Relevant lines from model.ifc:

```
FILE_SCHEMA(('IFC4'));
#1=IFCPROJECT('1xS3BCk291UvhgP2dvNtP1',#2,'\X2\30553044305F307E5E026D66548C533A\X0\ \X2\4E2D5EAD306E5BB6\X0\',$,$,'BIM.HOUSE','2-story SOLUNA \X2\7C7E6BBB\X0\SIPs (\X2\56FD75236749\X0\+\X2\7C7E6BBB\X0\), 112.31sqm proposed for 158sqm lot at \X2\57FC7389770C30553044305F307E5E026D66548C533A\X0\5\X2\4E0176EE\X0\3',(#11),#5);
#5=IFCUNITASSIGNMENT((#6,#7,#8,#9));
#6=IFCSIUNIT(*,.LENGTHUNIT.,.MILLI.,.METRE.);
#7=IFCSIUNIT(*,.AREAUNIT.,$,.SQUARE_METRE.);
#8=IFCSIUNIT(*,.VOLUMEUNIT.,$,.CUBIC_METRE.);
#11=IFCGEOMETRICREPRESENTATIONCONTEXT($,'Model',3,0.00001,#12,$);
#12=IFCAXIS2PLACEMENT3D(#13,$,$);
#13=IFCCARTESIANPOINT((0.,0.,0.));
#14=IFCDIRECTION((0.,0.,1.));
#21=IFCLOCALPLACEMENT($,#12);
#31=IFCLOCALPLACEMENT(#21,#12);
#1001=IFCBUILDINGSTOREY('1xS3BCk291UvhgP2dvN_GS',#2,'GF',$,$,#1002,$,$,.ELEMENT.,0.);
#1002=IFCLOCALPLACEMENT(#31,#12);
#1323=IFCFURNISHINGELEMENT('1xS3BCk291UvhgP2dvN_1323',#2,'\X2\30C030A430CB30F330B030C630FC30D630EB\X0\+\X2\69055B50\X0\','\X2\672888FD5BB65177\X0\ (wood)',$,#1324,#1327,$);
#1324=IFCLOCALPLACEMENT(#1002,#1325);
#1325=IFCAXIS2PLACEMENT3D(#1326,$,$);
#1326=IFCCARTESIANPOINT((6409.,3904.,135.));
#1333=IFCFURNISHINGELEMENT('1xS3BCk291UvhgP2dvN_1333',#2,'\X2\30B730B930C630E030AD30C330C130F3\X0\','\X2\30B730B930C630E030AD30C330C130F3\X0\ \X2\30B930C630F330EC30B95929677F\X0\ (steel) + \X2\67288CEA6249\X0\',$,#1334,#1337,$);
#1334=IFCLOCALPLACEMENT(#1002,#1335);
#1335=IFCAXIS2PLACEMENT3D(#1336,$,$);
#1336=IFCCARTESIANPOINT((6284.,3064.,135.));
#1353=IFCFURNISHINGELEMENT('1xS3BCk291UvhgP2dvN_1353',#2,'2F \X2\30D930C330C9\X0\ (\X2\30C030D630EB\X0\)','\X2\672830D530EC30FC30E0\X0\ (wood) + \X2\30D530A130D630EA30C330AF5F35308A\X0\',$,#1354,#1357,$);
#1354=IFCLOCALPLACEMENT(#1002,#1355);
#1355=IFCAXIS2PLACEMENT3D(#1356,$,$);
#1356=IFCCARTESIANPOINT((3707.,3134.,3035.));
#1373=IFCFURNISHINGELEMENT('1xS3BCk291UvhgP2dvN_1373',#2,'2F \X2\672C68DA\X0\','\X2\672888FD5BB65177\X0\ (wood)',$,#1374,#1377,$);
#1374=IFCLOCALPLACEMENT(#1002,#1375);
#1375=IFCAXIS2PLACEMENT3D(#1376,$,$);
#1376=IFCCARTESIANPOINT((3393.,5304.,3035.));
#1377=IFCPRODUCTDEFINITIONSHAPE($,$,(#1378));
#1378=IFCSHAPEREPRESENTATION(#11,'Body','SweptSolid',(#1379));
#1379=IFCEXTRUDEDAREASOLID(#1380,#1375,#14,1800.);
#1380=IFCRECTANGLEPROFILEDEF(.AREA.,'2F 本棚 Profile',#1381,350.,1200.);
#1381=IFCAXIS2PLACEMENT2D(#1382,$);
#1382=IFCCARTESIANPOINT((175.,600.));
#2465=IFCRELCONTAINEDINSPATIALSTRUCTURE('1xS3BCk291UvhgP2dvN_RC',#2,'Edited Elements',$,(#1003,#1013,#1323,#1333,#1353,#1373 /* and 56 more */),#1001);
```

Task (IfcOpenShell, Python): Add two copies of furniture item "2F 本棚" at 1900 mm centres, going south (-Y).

```python
import numpy as np
import ifcopenshell
import ifcopenshell.api.geometry
import ifcopenshell.api.root
import ifcopenshell.util.element
import ifcopenshell.util.placement
import ifcopenshell.util.unit

model = ifcopenshell.open("model.ifc")
unit_scale = ifcopenshell.util.unit.calculate_unit_scale(model)


def reuse_history(source, copy):
    """copy_class also copies each property set's owner history, people and application; keep the originals."""
    for rel in copy.IsDefinedBy:
        if rel.is_a("IfcRelDefinesByProperties") and (history := rel.RelatingPropertyDefinition.OwnerHistory):
            rel.RelatingPropertyDefinition.OwnerHistory = source.OwnerHistory
            ifcopenshell.util.element.remove_deep2(model, history)


source = model.by_id(1373)
base = ifcopenshell.util.placement.get_local_placement(source.ObjectPlacement)
step = np.array([0.0, -1.0, 0.0]) * 1.9 / unit_scale

for i in range(1, 3):
    copy = ifcopenshell.api.root.copy_class(model, product=source)
    copy.Representation = ifcopenshell.util.element.copy_deep(
        model, source.Representation, exclude=["IfcGeometricRepresentationContext", "IfcRepresentationMap"]
    )
    reuse_history(source, copy)
    matrix = base.copy()
    matrix[:3, 3] += i * step
    print("added at", matrix[:3, 3].round(3) + 0.0)
    ifcopenshell.api.geometry.edit_object_placement(model, product=copy, matrix=matrix, is_si=False)

model.write("model_v2.ifc")
```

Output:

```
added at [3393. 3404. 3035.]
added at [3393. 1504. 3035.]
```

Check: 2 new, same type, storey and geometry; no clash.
